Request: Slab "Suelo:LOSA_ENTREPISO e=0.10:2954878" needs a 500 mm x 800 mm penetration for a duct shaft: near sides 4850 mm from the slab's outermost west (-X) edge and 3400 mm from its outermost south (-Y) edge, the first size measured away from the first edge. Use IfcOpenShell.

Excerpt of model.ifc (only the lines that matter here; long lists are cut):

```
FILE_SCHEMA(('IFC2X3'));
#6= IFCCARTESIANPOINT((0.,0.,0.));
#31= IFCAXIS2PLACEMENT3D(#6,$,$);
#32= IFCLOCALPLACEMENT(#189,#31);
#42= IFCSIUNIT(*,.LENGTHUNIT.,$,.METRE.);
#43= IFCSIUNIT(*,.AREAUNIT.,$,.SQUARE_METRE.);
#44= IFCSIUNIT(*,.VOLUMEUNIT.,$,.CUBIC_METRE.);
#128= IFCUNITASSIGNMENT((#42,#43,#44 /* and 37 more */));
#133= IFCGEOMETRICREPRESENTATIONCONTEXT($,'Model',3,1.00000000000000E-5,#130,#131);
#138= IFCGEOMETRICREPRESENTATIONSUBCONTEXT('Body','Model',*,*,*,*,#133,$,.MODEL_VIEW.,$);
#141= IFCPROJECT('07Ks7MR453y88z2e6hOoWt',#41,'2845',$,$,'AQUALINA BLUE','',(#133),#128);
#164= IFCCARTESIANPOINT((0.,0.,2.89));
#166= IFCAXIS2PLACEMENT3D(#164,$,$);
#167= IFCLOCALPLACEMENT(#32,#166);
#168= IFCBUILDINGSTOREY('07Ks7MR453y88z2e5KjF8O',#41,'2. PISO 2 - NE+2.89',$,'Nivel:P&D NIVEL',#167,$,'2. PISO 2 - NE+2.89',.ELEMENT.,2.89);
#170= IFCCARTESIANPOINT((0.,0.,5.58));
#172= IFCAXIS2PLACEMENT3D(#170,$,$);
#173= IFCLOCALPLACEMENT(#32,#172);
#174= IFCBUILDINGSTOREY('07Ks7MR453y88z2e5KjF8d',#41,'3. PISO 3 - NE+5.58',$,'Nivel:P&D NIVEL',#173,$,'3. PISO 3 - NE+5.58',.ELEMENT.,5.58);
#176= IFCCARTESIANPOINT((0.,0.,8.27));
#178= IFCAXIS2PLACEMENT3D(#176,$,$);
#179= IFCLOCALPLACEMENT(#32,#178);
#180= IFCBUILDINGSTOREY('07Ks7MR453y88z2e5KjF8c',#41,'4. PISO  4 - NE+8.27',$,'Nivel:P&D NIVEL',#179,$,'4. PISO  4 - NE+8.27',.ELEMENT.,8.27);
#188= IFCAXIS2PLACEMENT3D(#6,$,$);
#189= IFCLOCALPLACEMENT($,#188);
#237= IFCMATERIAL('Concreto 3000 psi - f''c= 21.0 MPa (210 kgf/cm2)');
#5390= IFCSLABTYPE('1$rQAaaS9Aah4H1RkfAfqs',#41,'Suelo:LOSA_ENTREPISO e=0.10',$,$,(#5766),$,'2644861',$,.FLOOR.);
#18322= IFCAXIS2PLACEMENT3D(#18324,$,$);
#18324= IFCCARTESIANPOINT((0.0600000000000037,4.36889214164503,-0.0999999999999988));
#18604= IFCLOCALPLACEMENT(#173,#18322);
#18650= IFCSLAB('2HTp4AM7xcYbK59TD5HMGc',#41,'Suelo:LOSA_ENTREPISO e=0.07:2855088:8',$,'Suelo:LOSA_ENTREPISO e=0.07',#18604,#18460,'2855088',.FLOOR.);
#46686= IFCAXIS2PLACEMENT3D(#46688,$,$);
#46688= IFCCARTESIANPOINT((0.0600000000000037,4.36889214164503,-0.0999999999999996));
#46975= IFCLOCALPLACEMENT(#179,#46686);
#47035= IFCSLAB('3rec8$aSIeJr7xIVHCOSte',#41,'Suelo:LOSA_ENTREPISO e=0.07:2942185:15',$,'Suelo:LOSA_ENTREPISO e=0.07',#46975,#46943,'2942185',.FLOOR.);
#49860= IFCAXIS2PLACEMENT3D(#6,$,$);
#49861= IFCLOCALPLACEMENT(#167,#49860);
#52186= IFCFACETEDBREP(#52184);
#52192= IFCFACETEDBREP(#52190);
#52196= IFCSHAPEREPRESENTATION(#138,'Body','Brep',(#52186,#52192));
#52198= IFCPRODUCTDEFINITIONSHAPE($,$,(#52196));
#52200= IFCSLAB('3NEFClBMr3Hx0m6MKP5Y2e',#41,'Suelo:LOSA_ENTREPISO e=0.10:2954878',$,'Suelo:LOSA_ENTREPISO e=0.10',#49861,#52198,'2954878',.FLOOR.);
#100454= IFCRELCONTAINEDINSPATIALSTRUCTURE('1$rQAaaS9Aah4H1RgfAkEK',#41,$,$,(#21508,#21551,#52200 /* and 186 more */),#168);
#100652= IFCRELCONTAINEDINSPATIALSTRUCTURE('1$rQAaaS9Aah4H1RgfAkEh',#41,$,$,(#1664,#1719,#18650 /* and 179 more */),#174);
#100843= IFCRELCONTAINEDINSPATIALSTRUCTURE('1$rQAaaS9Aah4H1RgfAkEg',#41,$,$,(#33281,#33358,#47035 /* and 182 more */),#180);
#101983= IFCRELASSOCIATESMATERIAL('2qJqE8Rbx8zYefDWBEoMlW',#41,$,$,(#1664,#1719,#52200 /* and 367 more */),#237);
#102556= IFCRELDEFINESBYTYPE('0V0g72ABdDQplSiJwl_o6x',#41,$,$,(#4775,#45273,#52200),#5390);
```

```python
import numpy as np
import ifcopenshell
import ifcopenshell.api.feature
import ifcopenshell.api.geometry
import ifcopenshell.api.root
import ifcopenshell.geom
import ifcopenshell.util.placement
import ifcopenshell.util.representation
import ifcopenshell.util.shape
import ifcopenshell.util.unit

model = ifcopenshell.open("model.ifc")
unit_scale = ifcopenshell.util.unit.calculate_unit_scale(model)
settings = ifcopenshell.geom.settings()


def volume(element):
    """Net volume in cubic metres, openings subtracted."""
    shape = ifcopenshell.geom.create_shape(settings, element)
    return ifcopenshell.util.shape.get_volume(shape.geometry)


slab = model.by_guid("3NEFClBMr3Hx0m6MKP5Y2e")
before = volume(slab)

# Extent in the slab's own axes, in metres. The edges named are its -X and -Y sides.
slab_shape = ifcopenshell.geom.create_shape(settings, slab)
vertices = ifcopenshell.util.shape.get_vertices(slab_shape.geometry)
x_min, y_min, bottom = vertices.min(axis=0)
top = vertices[:, 2].max()

opening = ifcopenshell.api.root.create_entity(model, ifc_class="IfcOpeningElement", name="Duct shaft opening")
context = ifcopenshell.util.representation.get_context(model, "Model", "Body", "MODEL_VIEW")
width, depth = 0.5, 0.8
outline = [(0.0, 0.0), (width, 0.0), (width, depth), (0.0, depth), (0.0, 0.0)]
# Overshoot both faces by 50 mm so the cut is clean.
shape = ifcopenshell.api.geometry.add_slab_representation(
    model, context=context, depth=top - bottom + 0.1, polyline=outline
)
ifcopenshell.api.geometry.assign_representation(model, product=opening, representation=shape)

matrix = ifcopenshell.util.placement.get_local_placement(slab.ObjectPlacement)
matrix[:, 3] = matrix @ np.append(np.array([x_min + 4.85, y_min + 3.4, bottom - 0.05]) / unit_scale, 1.0)
ifcopenshell.api.geometry.edit_object_placement(model, product=opening, matrix=matrix, is_si=False)
ifcopenshell.api.feature.add_feature(model, feature=opening, element=slab)

after = volume(slab)

print(f"slab volume {before:.3f} -> {after:.3f} m3")

model.write("model-out.ifc")
```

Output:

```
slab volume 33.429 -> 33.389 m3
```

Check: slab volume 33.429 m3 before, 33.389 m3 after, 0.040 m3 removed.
